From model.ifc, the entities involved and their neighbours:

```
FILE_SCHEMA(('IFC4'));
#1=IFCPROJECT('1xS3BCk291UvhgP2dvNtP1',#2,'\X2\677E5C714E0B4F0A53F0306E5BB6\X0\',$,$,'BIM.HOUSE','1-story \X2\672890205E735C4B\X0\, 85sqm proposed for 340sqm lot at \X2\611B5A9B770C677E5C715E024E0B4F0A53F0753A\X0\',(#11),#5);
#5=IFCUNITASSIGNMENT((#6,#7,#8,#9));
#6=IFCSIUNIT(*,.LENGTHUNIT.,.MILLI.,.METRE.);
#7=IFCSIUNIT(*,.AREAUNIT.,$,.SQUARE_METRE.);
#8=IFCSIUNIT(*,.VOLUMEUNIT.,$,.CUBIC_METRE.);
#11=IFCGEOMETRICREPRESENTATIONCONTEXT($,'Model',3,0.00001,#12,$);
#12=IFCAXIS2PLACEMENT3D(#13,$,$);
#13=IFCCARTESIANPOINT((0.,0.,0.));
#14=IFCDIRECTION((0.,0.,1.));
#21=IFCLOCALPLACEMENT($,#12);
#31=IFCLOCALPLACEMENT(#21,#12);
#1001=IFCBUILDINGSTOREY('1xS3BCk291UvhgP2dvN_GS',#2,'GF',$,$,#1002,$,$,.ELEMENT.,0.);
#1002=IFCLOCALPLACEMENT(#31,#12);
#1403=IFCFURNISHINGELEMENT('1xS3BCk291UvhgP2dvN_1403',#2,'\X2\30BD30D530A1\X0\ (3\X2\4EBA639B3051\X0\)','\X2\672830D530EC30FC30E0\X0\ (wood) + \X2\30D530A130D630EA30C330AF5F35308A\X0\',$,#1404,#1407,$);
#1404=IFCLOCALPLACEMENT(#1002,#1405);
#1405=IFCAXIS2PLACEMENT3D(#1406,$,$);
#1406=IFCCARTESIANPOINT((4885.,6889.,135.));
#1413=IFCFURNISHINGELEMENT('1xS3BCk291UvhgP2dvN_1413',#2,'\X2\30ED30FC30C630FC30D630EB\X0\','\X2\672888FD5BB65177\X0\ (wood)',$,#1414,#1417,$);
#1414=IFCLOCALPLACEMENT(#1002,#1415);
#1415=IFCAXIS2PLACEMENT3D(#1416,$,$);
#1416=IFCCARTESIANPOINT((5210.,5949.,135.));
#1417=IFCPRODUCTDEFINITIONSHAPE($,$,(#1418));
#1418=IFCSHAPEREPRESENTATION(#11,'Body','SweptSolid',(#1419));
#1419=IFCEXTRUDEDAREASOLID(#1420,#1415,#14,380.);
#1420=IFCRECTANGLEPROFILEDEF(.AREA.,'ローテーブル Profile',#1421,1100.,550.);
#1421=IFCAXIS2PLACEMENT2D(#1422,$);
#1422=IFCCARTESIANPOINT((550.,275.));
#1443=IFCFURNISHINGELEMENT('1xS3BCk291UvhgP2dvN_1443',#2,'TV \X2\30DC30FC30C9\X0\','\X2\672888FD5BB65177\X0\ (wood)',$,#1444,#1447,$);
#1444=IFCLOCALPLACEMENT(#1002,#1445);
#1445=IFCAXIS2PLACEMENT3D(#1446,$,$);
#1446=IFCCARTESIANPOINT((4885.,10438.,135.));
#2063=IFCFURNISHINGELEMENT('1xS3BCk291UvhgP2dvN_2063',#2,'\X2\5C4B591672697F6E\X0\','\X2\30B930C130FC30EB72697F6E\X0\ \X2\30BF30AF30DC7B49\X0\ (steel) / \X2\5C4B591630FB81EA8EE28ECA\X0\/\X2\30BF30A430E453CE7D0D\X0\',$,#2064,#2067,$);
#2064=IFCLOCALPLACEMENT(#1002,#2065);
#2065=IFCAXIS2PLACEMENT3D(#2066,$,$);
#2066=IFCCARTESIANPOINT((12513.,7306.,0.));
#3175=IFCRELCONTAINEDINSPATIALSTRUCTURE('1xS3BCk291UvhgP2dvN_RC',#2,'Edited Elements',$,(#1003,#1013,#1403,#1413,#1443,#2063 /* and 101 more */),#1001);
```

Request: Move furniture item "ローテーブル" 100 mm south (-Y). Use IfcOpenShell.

```python
import ifcopenshell
import ifcopenshell.api.geometry
import ifcopenshell.util.placement

model = ifcopenshell.open("model.ifc")

item = model.by_id(1413)
matrix = ifcopenshell.util.placement.get_local_placement(item.ObjectPlacement)
matrix[1, 3] -= 100.0
ifcopenshell.api.geometry.edit_object_placement(model, product=item, matrix=matrix, is_si=False)

print(ifcopenshell.util.placement.get_local_placement(item.ObjectPlacement).round(3) + 0.0)

model.write("model_rev.ifc")
```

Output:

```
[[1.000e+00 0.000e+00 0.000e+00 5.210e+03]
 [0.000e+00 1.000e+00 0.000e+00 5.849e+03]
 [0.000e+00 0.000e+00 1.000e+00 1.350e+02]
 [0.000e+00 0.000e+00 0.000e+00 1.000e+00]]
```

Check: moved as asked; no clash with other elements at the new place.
